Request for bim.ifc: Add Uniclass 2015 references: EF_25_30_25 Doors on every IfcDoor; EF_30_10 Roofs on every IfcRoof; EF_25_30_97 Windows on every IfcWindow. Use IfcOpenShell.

First a look at what the model holds.

```python
import ifcopenshell

model = ifcopenshell.open("bim.ifc")
print(model.schema)
print("classifications:", [c.Name for c in model.by_type("IfcClassification")])
for ifc_class in ("IfcDoor", "IfcRoof", "IfcStair", "IfcWall", "IfcWindow"):
    print(ifc_class, len(model.by_type(ifc_class)))
```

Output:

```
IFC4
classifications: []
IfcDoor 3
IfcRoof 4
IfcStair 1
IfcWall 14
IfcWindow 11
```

```python
import ifcopenshell
import ifcopenshell.api.classification

model = ifcopenshell.open("bim.ifc")

system = ifcopenshell.api.classification.add_classification(model, classification="Uniclass 2015")

codes = {
    "IfcDoor": ("EF_25_30_25", "Doors"),
    "IfcRoof": ("EF_30_10", "Roofs"),
    "IfcWindow": ("EF_25_30_97", "Windows"),
}
for ifc_class, (code, name) in codes.items():
    products = model.by_type(ifc_class)
    ifcopenshell.api.classification.add_reference(
        model, products=products, classification=system, identification=code, name=name
    )
    print(code, len(products))

model.write("bim-out.ifc")
```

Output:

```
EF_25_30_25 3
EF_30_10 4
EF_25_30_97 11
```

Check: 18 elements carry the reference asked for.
